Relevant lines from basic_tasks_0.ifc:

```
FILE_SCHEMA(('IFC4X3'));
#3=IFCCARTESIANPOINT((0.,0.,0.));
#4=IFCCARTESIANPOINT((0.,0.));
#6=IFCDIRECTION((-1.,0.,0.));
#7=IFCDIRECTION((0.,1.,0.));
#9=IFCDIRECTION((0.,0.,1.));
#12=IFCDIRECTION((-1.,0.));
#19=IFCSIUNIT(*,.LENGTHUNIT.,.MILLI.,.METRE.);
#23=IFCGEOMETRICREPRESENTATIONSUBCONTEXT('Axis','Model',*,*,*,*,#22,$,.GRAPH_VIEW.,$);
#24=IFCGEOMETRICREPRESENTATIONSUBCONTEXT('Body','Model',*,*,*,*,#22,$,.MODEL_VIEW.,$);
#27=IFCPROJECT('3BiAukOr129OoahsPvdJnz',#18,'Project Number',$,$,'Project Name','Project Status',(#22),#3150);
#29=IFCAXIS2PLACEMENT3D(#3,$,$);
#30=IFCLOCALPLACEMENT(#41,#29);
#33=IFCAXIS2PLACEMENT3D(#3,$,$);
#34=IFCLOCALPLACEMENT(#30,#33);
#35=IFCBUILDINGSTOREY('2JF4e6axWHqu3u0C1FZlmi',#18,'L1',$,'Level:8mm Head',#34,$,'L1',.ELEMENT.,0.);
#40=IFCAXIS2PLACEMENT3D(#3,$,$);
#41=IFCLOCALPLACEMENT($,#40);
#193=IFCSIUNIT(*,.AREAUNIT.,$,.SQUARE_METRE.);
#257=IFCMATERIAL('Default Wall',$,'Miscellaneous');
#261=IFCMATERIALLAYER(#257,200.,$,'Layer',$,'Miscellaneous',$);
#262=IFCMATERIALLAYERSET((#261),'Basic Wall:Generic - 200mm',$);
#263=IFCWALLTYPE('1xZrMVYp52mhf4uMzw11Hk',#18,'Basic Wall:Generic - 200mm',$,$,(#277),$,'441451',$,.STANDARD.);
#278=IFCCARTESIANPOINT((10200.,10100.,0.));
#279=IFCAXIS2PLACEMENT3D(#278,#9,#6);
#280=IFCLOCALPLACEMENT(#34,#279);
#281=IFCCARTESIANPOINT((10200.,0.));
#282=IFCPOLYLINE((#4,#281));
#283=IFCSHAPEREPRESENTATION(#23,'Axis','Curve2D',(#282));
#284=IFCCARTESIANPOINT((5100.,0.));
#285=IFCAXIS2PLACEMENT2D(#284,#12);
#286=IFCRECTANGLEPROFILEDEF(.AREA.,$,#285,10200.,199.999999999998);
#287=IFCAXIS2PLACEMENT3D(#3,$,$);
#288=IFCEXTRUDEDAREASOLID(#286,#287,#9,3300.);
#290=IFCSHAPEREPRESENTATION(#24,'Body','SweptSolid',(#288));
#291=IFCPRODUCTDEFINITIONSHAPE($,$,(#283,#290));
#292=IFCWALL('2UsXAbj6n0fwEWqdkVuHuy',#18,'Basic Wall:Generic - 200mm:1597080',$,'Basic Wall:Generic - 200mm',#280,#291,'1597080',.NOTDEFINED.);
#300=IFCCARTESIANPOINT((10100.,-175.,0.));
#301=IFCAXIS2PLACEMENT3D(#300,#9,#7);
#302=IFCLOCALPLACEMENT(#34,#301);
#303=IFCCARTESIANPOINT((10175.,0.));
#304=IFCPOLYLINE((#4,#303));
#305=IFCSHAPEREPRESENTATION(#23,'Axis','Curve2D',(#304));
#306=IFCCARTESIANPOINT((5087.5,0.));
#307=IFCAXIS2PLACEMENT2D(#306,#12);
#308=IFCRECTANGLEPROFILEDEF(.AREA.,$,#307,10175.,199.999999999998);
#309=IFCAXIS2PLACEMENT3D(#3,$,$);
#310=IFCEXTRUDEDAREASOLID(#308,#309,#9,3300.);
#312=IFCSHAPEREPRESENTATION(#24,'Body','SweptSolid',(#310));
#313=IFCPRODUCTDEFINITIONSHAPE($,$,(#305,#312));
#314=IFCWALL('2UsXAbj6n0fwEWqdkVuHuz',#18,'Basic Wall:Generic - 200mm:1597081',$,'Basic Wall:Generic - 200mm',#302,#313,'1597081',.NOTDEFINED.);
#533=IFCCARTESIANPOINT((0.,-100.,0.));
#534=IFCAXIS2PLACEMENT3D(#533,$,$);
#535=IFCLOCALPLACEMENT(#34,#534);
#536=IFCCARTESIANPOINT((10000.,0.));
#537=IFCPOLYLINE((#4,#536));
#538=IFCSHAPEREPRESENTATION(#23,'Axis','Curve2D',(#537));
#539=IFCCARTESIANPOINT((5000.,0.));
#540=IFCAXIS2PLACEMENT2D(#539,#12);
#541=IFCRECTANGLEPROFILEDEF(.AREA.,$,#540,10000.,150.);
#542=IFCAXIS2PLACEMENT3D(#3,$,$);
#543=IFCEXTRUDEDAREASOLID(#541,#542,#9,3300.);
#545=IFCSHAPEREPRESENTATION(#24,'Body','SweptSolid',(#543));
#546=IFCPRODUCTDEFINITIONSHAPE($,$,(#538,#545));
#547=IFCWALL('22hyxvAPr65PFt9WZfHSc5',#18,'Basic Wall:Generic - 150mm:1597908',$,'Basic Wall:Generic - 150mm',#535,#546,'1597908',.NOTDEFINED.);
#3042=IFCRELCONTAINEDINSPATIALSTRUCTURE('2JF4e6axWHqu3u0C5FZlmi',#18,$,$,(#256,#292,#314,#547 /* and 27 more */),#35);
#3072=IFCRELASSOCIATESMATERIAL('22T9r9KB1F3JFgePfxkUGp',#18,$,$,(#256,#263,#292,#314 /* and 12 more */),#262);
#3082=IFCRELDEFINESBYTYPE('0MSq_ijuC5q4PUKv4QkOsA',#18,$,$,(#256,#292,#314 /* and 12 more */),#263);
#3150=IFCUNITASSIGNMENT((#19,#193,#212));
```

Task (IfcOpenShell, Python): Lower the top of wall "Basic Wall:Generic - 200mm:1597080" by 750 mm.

```python
import ifcopenshell
import ifcopenshell.geom
import ifcopenshell.util.representation
import ifcopenshell.util.shape
import ifcopenshell.util.unit

model = ifcopenshell.open("basic_tasks_0.ifc")
unit_scale = ifcopenshell.util.unit.calculate_unit_scale(model)
settings = ifcopenshell.geom.settings()


def volume(element):
    """Net volume in cubic metres, openings subtracted."""
    shape = ifcopenshell.geom.create_shape(settings, element)
    return ifcopenshell.util.shape.get_volume(shape.geometry)


wall = model.by_id(292)
before = volume(wall)

body = ifcopenshell.util.representation.get_representation(wall, "Model", "Body")
solid = body.Items[0]
old_height = solid.Depth
solid.Depth -= 0.75 / unit_scale
after = volume(wall)

print(f"height {old_height:g} -> {solid.Depth:g}, volume {before:.3f} -> {after:.3f} m3")

model.write("basic_tasks_0_edited.ifc")
```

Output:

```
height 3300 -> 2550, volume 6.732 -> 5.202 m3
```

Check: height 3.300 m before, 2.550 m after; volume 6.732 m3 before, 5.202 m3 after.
